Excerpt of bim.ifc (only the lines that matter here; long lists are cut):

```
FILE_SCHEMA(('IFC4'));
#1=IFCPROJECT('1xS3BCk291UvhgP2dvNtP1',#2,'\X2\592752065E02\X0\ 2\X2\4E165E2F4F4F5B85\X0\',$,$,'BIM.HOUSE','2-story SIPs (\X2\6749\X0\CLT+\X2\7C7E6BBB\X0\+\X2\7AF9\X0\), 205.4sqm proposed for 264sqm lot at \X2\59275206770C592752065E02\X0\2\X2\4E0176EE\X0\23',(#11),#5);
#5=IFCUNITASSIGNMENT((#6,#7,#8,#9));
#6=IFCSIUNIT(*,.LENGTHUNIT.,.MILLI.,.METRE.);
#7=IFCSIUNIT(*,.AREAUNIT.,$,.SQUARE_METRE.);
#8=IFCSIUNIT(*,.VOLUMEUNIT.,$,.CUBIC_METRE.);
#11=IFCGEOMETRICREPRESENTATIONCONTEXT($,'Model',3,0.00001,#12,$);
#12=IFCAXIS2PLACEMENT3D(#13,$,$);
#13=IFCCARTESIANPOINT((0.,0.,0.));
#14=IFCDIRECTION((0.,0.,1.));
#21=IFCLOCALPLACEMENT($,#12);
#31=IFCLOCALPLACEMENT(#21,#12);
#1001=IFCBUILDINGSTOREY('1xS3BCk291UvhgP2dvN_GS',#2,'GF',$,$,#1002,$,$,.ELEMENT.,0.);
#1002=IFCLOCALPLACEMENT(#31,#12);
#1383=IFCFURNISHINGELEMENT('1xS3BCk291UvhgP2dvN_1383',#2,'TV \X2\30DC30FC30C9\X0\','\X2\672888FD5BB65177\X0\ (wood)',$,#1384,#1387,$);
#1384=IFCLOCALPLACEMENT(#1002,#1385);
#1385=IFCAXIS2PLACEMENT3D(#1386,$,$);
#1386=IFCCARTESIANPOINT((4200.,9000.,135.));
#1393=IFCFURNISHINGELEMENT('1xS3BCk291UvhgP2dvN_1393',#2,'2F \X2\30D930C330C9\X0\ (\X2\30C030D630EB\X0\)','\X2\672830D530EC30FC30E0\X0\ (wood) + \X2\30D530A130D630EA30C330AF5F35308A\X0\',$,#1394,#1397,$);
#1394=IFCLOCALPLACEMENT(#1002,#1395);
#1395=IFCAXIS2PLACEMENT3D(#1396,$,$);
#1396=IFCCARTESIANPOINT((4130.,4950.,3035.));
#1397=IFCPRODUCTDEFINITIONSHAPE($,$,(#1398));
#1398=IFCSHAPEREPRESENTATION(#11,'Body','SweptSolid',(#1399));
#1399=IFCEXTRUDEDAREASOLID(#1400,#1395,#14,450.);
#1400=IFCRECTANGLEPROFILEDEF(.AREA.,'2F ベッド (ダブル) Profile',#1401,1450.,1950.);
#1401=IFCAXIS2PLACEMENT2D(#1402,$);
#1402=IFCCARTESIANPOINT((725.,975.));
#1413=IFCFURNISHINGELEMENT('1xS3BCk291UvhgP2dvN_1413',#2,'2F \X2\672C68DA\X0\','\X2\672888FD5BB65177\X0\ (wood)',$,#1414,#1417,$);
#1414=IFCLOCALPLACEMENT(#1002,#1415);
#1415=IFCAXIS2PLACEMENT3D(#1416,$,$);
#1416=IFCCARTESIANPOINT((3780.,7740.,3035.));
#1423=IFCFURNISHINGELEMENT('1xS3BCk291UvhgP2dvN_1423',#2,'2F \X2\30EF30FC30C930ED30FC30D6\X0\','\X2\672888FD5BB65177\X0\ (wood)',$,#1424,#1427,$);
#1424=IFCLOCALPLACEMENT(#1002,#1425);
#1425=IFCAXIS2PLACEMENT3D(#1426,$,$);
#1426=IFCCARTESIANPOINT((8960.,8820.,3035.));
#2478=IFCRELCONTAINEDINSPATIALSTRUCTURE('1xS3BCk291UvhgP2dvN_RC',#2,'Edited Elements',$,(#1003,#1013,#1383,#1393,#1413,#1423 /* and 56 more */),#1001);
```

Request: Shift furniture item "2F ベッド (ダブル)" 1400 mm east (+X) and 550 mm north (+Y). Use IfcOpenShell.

```python
import ifcopenshell
import ifcopenshell.api.geometry
import ifcopenshell.util.placement
import ifcopenshell.util.unit

model = ifcopenshell.open("bim.ifc")
unit_scale = ifcopenshell.util.unit.calculate_unit_scale(model)

item = model.by_guid("1xS3BCk291UvhgP2dvN_1393")
matrix = ifcopenshell.util.placement.get_local_placement(item.ObjectPlacement)
matrix[0, 3] += 1.4 / unit_scale
matrix[1, 3] += 0.55 / unit_scale
ifcopenshell.api.geometry.edit_object_placement(model, product=item, matrix=matrix, is_si=False)

print(ifcopenshell.util.placement.get_local_placement(item.ObjectPlacement).round(3) + 0.0)

model.write("bim-out.ifc")
```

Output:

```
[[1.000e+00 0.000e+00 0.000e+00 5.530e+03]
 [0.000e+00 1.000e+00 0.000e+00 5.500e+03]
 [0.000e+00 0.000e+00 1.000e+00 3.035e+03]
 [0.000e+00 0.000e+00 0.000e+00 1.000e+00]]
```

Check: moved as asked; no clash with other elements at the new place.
